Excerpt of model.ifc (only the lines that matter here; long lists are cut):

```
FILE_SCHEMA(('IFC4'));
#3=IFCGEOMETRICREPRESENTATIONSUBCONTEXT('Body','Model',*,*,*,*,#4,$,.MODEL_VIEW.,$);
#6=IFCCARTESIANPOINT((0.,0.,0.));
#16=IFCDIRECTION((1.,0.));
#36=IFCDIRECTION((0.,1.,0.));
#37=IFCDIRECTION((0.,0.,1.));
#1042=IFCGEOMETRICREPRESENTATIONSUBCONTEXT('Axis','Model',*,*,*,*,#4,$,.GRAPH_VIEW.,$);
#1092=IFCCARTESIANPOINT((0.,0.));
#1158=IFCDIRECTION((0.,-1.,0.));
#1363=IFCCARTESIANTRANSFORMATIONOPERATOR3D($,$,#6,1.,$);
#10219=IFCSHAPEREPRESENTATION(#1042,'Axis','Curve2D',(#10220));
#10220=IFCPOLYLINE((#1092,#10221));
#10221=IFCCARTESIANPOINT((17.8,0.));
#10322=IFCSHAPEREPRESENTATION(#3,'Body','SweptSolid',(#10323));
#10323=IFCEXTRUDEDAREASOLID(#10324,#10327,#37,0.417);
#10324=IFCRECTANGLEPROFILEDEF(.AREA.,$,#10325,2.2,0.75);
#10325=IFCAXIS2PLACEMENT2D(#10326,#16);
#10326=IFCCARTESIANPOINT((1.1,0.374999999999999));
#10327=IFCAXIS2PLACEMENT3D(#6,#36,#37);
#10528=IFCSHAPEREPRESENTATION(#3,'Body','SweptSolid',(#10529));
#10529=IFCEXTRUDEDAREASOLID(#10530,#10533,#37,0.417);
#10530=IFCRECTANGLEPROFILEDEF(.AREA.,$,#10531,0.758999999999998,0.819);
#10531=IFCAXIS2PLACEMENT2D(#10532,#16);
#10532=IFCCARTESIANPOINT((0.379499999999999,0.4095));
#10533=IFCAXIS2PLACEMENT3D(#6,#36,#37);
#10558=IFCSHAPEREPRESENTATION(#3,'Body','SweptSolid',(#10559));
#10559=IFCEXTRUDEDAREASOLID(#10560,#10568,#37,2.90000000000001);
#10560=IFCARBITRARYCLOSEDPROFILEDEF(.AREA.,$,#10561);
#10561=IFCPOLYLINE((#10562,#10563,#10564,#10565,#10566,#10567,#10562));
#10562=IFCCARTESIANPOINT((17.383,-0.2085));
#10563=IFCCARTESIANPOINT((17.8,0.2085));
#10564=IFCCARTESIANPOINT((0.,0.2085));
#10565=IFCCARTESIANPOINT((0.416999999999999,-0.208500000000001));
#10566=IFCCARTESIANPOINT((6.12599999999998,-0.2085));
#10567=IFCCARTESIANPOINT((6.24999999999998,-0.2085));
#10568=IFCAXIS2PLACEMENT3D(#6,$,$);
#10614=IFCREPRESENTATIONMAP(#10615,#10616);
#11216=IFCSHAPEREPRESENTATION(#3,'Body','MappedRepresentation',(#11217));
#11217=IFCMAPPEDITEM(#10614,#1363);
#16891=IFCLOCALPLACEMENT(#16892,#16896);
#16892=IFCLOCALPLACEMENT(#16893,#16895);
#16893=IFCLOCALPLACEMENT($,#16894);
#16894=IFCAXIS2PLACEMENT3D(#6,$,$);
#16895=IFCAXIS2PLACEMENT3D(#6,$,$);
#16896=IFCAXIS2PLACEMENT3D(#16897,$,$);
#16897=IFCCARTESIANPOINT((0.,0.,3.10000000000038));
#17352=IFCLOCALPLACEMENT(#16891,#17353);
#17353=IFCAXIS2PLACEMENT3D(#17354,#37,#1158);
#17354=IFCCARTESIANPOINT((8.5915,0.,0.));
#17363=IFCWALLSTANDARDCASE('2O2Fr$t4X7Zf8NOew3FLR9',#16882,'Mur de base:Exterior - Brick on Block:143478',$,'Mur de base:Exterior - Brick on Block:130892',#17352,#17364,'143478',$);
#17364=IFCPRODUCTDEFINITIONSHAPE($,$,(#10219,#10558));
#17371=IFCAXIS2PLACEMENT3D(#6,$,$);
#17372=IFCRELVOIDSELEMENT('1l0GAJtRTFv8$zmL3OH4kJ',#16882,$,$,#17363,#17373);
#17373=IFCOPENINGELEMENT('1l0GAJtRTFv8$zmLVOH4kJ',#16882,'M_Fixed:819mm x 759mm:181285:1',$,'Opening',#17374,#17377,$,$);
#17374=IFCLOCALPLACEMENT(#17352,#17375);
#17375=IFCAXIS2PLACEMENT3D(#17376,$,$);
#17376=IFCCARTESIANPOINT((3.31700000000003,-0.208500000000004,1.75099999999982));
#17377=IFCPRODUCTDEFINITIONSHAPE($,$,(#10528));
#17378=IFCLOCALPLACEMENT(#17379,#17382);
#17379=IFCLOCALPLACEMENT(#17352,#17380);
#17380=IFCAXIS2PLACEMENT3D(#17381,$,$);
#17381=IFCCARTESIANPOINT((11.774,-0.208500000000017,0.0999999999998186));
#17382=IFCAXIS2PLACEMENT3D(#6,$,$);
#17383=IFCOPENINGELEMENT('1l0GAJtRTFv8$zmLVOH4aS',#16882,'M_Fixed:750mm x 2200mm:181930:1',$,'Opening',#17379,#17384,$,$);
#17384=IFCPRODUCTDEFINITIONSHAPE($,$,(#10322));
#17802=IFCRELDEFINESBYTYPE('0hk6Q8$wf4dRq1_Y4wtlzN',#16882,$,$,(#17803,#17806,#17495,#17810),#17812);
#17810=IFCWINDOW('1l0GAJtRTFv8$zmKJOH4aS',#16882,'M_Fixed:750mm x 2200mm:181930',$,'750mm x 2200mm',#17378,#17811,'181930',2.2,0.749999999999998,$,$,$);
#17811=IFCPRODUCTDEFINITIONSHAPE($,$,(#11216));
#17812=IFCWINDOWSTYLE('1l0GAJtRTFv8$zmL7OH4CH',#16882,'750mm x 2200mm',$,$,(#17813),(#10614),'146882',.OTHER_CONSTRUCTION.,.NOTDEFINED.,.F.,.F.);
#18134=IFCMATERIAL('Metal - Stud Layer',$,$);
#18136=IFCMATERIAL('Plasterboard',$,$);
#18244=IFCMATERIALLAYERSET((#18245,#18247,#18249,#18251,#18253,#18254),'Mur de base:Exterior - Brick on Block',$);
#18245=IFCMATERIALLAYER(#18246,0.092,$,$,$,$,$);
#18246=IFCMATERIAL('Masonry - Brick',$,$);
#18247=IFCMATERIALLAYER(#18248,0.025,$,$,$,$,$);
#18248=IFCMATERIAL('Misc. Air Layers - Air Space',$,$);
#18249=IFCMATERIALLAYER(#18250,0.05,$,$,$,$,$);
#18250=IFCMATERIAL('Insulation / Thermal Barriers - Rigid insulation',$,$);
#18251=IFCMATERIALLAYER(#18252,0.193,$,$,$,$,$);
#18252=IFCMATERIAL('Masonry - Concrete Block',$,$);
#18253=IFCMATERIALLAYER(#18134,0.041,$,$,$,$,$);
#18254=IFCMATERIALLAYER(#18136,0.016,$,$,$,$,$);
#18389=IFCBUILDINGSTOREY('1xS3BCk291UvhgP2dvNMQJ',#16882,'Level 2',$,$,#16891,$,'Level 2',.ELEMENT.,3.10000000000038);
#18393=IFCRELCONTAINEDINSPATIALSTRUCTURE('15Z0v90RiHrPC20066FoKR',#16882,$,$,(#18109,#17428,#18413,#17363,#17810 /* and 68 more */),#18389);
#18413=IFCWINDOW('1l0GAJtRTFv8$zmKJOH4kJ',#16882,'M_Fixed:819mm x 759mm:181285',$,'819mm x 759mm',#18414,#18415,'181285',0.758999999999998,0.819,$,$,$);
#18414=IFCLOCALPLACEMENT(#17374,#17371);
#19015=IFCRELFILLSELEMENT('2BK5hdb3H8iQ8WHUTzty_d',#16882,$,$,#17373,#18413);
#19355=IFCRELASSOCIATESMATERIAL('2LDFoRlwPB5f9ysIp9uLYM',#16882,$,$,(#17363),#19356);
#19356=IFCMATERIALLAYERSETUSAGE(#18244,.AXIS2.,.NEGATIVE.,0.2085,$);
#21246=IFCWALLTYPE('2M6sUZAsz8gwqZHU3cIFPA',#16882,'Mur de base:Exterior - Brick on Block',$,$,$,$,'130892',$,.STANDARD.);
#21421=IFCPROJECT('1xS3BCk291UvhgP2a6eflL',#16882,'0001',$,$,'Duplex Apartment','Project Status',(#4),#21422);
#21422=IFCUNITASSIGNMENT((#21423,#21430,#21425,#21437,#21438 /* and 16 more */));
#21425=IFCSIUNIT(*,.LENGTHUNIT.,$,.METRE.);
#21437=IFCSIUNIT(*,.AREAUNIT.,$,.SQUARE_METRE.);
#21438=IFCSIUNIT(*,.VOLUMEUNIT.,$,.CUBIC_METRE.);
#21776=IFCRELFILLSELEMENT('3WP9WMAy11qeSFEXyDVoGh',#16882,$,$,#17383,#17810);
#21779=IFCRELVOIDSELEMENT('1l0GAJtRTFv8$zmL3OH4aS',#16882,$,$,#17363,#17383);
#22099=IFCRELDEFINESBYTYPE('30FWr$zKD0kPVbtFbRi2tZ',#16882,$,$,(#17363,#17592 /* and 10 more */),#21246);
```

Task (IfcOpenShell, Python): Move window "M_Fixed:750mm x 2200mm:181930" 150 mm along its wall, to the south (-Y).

```python
import ifcopenshell
import ifcopenshell.api.geometry
import ifcopenshell.util.placement
import ifcopenshell.util.unit

model = ifcopenshell.open("model.ifc")
unit_scale = ifcopenshell.util.unit.calculate_unit_scale(model)

window = model.by_id(17810)
opening = window.FillsVoids[0].RelatingOpeningElement
wall = opening.VoidsElements[0].RelatingBuildingElement

wall_matrix = ifcopenshell.util.placement.get_local_placement(wall.ObjectPlacement)
shift = wall_matrix[:3, 0] * 0.15 / unit_scale
before = ifcopenshell.util.placement.get_local_placement(window.ObjectPlacement)[:3, 3].copy()

# The window is placed relative to its opening, so it follows when the opening moves.
matrix = ifcopenshell.util.placement.get_local_placement(opening.ObjectPlacement)
matrix[:3, 3] += shift
ifcopenshell.api.geometry.edit_object_placement(
    model, product=opening, matrix=matrix, is_si=False, should_transform_children=True
)

after = ifcopenshell.util.placement.get_local_placement(window.ObjectPlacement)[:3, 3]
print("window moved by", (after - before).round(3) + 0.0)

model.write("model_rev.ifc")
```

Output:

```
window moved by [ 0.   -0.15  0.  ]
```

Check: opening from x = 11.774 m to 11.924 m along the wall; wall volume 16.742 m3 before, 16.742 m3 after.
